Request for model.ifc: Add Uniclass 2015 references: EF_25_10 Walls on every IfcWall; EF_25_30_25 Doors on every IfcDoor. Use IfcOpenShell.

First a look at what the model holds.

```python
import ifcopenshell

model = ifcopenshell.open("model.ifc")
print(model.schema)
print("classifications:", [c.Name for c in model.by_type("IfcClassification")])
for ifc_class in ("IfcDoor", "IfcRoof", "IfcStair", "IfcWall", "IfcWindow"):
    print(ifc_class, len(model.by_type(ifc_class)))
```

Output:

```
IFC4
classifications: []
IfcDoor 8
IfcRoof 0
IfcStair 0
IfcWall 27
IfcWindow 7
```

```python
import ifcopenshell
import ifcopenshell.api.classification

model = ifcopenshell.open("model.ifc")

system = ifcopenshell.api.classification.add_classification(model, classification="Uniclass 2015")

codes = {
    "IfcWall": ("EF_25_10", "Walls"),
    "IfcDoor": ("EF_25_30_25", "Doors"),
}
for ifc_class, (code, name) in codes.items():
    products = model.by_type(ifc_class)
    ifcopenshell.api.classification.add_reference(
        model, products=products, classification=system, identification=code, name=name
    )
    print(code, len(products))

model.write("model_updated.ifc")
```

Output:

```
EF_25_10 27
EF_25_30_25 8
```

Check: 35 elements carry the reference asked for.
